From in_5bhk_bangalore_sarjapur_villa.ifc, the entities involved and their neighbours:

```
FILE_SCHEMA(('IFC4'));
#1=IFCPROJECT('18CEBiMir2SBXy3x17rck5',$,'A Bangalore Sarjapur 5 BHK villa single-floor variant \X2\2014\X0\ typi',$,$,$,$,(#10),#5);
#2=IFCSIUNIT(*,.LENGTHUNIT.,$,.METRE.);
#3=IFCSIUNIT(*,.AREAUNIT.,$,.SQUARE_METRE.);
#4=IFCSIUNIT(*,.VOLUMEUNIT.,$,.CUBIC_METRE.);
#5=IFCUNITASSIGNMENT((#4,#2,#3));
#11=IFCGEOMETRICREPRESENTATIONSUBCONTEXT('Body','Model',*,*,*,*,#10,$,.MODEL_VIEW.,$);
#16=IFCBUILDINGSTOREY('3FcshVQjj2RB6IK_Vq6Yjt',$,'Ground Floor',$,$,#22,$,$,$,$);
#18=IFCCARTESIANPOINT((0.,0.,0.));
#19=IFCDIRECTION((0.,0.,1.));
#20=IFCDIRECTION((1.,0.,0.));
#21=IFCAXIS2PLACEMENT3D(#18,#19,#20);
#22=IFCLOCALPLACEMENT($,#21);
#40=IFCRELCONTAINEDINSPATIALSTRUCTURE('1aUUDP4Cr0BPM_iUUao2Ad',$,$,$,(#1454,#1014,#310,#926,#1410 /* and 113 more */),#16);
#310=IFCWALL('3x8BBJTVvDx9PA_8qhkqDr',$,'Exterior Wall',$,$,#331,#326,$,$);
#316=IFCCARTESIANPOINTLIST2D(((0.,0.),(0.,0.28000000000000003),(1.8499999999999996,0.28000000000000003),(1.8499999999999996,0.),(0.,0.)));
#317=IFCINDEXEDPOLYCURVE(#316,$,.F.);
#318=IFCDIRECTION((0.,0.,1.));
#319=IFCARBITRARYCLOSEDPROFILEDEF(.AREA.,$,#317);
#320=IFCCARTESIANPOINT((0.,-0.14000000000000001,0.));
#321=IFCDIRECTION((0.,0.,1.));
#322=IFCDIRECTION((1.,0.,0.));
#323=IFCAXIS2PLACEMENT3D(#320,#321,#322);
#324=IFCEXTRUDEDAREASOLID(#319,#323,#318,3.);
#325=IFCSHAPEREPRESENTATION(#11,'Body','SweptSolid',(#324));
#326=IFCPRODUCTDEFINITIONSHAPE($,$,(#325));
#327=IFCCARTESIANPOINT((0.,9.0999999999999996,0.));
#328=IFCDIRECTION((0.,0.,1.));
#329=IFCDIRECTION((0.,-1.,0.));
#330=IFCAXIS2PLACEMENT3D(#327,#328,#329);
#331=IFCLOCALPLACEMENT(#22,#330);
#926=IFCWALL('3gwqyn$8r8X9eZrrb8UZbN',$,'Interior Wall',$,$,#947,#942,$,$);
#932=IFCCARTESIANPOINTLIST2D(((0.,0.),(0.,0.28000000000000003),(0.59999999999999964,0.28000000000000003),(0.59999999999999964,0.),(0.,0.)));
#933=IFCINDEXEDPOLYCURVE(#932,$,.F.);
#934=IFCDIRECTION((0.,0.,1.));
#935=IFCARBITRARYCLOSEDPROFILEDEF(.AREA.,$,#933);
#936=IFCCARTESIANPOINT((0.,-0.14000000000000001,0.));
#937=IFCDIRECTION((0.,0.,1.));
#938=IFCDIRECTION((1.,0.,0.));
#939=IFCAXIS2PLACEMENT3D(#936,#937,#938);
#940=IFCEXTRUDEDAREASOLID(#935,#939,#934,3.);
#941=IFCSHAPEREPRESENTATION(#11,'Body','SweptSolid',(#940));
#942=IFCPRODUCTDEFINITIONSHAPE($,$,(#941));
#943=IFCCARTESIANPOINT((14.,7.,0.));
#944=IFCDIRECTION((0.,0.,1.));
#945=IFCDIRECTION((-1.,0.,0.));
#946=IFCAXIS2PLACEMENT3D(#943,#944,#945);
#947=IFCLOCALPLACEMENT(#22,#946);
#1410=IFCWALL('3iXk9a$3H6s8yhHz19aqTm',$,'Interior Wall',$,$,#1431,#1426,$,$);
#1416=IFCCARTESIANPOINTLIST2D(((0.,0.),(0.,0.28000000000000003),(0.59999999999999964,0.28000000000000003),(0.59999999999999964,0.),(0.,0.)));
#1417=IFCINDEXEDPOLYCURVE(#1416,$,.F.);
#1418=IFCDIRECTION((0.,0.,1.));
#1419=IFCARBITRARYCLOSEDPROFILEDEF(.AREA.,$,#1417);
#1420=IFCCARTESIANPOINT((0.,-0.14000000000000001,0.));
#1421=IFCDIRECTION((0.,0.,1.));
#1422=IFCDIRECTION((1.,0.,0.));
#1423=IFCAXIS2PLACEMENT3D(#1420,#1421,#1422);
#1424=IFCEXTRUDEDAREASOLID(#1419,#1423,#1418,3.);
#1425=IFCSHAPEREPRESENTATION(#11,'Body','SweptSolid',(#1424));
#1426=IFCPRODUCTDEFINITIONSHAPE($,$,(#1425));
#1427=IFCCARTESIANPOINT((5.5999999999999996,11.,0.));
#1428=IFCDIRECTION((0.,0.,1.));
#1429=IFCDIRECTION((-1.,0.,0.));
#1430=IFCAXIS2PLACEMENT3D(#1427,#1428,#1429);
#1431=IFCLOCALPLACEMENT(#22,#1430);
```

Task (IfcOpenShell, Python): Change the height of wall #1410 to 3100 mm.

```python
import ifcopenshell
import ifcopenshell.geom
import ifcopenshell.util.representation
import ifcopenshell.util.shape
import ifcopenshell.util.unit

model = ifcopenshell.open("in_5bhk_bangalore_sarjapur_villa.ifc")
unit_scale = ifcopenshell.util.unit.calculate_unit_scale(model)
settings = ifcopenshell.geom.settings()


def volume(element):
    """Net volume in cubic metres, openings subtracted."""
    shape = ifcopenshell.geom.create_shape(settings, element)
    return ifcopenshell.util.shape.get_volume(shape.geometry)


wall = model.by_guid("3iXk9a$3H6s8yhHz19aqTm")
before = volume(wall)

body = ifcopenshell.util.representation.get_representation(wall, "Model", "Body")
solid = body.Items[0]
old_height = solid.Depth
solid.Depth = 3.1 / unit_scale
after = volume(wall)

print(f"height {old_height:g} -> {solid.Depth:g}, volume {before:.3f} -> {after:.3f} m3")

model.write("in_5bhk_bangalore_sarjapur_villa_updated.ifc")
```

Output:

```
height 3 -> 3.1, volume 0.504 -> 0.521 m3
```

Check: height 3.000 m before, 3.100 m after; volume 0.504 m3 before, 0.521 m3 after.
